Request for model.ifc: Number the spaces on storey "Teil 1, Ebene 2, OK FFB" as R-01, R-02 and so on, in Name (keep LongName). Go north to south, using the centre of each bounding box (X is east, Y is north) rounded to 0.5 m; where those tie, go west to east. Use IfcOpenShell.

First a look at what the model holds.

```python
import ifcopenshell
import ifcopenshell.util.element
import ifcopenshell.util.placement

model = ifcopenshell.open("model.ifc")
print(model.schema)
storey = next(s for s in model.by_type("IfcBuildingStorey") if s.Name == "Teil 1, Ebene 2, OK FFB")
spaces = [e for e in ifcopenshell.util.element.get_decomposition(storey) if e.is_a("IfcSpace")]
for e in sorted(spaces, key=lambda e: e.id()):
    origin = ifcopenshell.util.placement.get_local_placement(e.ObjectPlacement)[:3, 3]
    print(e.id(), e.Name, e.LongName, origin.round(2) + 0.0, sep=" | ")
```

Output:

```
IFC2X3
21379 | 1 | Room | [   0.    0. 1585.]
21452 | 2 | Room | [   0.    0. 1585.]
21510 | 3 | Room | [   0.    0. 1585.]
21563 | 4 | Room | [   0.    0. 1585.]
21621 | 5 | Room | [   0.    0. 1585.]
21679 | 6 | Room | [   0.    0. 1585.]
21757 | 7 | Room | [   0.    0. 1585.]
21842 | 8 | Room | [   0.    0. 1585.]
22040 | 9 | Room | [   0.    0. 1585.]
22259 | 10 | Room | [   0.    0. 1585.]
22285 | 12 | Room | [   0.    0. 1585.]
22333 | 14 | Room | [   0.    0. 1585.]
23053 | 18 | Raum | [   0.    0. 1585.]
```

```python
import ifcopenshell
import ifcopenshell.geom
import ifcopenshell.util.element
import ifcopenshell.util.shape

model = ifcopenshell.open("model.ifc")
settings = ifcopenshell.geom.settings()
settings.set("use-world-coords", True)


def centre(element):
    shape = ifcopenshell.geom.create_shape(settings, element)
    return ifcopenshell.util.shape.get_bbox_centroid(shape.geometry)


storey = next(s for s in model.by_type("IfcBuildingStorey") if s.Name == "Teil 1, Ebene 2, OK FFB")
spaces = [e for e in ifcopenshell.util.element.get_decomposition(storey) if e.is_a("IfcSpace")]

# Insertion points can sit at a corner or the storey origin, so sort by the geometry (in metres).
centres = {e: centre(e) for e in spaces}
spaces.sort(key=lambda e: (-round(centres[e][1] / 0.5), centres[e][0]))

for i, e in enumerate(spaces, start=1):
    number = f"R-{i:02d}"
    e.Name = number
    print(e.id(), number)

model.write("model-out.ifc")
```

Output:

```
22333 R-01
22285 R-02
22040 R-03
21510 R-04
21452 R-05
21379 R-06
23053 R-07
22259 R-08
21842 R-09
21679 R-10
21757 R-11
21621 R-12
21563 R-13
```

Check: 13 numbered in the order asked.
